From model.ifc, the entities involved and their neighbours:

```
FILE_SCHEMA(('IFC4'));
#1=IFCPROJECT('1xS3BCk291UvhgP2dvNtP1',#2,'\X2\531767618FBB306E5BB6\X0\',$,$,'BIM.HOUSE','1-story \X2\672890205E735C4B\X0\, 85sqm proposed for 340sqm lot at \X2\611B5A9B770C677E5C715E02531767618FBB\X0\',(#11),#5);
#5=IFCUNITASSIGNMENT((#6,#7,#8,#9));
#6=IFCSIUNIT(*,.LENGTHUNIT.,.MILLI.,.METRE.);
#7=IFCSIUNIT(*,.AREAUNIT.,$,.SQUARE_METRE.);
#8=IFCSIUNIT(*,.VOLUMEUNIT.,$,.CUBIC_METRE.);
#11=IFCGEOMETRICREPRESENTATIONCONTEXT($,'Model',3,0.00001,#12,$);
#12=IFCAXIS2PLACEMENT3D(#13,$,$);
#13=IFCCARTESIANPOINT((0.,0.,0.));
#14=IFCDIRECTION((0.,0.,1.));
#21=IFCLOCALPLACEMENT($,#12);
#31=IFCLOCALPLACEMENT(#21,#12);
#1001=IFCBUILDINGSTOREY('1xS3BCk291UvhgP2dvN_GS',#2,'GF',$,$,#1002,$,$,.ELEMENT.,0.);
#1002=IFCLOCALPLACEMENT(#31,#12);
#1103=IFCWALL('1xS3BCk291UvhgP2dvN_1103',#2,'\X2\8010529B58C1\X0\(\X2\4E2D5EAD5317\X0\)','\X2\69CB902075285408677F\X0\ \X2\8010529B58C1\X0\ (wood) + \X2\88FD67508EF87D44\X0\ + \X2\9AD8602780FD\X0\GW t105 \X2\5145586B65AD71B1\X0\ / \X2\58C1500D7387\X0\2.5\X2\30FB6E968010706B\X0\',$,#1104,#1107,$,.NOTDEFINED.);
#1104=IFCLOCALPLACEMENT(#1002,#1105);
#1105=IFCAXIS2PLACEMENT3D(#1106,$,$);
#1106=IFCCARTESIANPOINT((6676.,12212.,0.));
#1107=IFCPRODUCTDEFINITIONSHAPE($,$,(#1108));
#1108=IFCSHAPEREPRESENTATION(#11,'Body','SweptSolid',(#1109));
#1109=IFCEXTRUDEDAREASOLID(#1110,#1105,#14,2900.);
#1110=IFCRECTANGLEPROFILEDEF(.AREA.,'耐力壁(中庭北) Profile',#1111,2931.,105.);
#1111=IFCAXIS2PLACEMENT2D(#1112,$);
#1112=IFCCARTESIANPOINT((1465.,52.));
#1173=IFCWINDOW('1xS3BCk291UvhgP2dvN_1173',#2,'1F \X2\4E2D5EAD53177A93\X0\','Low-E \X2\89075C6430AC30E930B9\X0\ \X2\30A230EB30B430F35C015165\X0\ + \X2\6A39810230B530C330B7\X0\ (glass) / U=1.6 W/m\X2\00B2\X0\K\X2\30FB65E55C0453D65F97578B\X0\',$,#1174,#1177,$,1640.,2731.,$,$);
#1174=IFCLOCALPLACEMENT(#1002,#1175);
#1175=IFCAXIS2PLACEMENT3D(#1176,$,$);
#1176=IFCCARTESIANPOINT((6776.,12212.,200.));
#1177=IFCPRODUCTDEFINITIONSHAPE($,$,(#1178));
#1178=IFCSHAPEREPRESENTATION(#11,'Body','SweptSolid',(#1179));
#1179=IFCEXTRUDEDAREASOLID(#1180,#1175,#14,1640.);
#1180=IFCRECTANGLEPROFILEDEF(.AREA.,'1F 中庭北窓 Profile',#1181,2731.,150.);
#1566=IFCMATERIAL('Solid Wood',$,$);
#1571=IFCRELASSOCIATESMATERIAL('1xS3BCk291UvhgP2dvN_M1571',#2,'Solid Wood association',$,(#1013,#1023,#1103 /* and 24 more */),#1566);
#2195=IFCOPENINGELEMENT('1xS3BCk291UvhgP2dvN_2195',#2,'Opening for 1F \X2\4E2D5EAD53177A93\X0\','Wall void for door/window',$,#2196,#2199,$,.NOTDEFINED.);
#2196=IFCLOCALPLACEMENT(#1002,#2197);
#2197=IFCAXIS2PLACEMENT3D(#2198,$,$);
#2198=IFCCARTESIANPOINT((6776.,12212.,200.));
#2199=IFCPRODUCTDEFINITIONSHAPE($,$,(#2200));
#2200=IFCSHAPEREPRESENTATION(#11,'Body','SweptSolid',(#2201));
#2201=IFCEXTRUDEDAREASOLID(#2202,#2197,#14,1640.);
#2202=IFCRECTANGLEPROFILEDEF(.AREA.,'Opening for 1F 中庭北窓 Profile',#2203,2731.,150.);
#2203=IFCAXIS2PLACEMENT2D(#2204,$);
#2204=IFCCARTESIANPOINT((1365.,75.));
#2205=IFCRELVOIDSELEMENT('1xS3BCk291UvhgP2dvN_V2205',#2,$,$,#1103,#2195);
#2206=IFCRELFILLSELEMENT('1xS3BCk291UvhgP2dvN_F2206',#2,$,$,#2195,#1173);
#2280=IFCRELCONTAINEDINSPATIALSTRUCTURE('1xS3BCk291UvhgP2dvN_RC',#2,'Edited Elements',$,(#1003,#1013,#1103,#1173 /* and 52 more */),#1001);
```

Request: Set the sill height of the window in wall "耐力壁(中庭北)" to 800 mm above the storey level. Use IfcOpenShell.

```python
import numpy as np
import ifcopenshell
import ifcopenshell.api.geometry
import ifcopenshell.geom
import ifcopenshell.util.element
import ifcopenshell.util.placement
import ifcopenshell.util.shape
import ifcopenshell.util.unit

model = ifcopenshell.open("model.ifc")
unit_scale = ifcopenshell.util.unit.calculate_unit_scale(model)

window = model.by_guid("1xS3BCk291UvhgP2dvN_1173")
opening = window.FillsVoids[0].RelatingOpeningElement
storey = ifcopenshell.util.element.get_container(window, ifc_class="IfcBuildingStorey")
level = ifcopenshell.util.placement.get_local_placement(storey.ObjectPlacement)[2, 3]

# The opening's origin need not be at the sill, so measure its lowest point.
shape = ifcopenshell.geom.create_shape(ifcopenshell.geom.settings(), opening)
bottom = ifcopenshell.util.shape.get_shape_bottom_elevation(shape, shape.geometry) / unit_scale
dz = level + 800.0 - bottom

shift = np.array([0.0, 0.0, dz])
# The window is not placed relative to its opening, so move both.
for product in (opening, window):
    matrix = ifcopenshell.util.placement.get_local_placement(product.ObjectPlacement)
    matrix[:3, 3] += shift
    ifcopenshell.api.geometry.edit_object_placement(model, product=product, matrix=matrix, is_si=False)

print(f"moved by {dz * unit_scale:+.3f} m")

model.write("model_rev.ifc")
```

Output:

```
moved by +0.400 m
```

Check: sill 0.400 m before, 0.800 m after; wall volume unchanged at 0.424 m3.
